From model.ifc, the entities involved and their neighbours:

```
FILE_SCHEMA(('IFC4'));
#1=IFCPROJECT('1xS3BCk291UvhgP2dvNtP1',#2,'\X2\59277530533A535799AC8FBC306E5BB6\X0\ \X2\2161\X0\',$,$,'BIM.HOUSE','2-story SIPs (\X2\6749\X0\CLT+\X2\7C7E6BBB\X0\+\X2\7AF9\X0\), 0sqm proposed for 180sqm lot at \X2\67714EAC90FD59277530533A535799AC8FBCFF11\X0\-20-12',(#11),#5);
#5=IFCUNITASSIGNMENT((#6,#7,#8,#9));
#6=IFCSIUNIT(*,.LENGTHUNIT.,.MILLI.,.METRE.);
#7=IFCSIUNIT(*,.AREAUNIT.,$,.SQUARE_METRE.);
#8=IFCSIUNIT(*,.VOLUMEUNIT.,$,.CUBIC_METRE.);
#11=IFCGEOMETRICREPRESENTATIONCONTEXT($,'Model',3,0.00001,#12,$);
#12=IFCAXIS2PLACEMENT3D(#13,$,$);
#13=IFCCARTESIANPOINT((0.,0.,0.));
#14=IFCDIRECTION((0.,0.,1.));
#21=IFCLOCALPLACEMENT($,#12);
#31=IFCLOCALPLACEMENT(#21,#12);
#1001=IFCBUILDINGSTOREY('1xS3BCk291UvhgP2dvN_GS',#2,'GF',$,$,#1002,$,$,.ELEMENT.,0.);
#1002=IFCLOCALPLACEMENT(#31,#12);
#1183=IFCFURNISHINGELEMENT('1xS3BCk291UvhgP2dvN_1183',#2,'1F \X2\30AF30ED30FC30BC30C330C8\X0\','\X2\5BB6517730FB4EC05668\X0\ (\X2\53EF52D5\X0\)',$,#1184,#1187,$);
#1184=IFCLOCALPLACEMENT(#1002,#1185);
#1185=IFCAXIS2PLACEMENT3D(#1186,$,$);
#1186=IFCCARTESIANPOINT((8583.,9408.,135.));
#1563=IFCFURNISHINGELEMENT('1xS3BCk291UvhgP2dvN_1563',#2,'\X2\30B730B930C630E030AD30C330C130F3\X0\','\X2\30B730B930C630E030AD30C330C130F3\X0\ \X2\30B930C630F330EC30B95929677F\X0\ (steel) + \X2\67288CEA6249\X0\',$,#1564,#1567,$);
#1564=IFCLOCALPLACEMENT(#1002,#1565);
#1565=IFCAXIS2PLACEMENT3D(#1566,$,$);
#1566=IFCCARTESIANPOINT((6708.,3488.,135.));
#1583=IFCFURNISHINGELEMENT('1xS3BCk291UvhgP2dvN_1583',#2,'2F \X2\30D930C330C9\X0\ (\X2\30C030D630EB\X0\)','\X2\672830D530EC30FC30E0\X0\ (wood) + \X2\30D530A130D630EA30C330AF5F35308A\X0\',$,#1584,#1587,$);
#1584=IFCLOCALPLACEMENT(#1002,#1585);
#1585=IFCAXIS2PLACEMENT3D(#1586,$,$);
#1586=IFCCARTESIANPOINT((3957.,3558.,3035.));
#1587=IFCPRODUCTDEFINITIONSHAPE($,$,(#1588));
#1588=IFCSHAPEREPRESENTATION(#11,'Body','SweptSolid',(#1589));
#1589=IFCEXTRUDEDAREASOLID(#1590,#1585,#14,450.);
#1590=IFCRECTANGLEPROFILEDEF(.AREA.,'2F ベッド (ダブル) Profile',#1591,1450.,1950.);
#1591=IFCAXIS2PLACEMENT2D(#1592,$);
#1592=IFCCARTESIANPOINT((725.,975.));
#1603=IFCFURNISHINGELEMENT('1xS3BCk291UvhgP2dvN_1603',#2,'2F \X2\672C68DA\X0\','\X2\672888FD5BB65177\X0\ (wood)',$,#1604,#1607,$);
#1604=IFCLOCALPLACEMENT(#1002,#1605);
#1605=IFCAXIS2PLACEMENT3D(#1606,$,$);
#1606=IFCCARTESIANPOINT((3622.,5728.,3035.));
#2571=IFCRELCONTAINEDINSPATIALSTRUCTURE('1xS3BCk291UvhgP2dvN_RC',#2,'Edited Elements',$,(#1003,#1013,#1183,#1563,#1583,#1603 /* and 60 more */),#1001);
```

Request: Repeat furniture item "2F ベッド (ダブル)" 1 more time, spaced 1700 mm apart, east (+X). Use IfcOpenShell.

```python
import numpy as np
import ifcopenshell
import ifcopenshell.api.geometry
import ifcopenshell.api.root
import ifcopenshell.util.element
import ifcopenshell.util.placement
import ifcopenshell.util.unit

model = ifcopenshell.open("model.ifc")
unit_scale = ifcopenshell.util.unit.calculate_unit_scale(model)


def reuse_history(source, copy):
    """copy_class also copies each property set's owner history, people and application; keep the originals."""
    for rel in copy.IsDefinedBy:
        if rel.is_a("IfcRelDefinesByProperties") and (history := rel.RelatingPropertyDefinition.OwnerHistory):
            rel.RelatingPropertyDefinition.OwnerHistory = source.OwnerHistory
            ifcopenshell.util.element.remove_deep2(model, history)


source = model.by_guid("1xS3BCk291UvhgP2dvN_1583")
base = ifcopenshell.util.placement.get_local_placement(source.ObjectPlacement)
step = np.array([1.0, 0.0, 0.0]) * 1.7 / unit_scale

for i in range(1, 2):
    copy = ifcopenshell.api.root.copy_class(model, product=source)
    copy.Representation = ifcopenshell.util.element.copy_deep(
        model, source.Representation, exclude=["IfcGeometricRepresentationContext", "IfcRepresentationMap"]
    )
    reuse_history(source, copy)
    matrix = base.copy()
    matrix[:3, 3] += i * step
    print("added at", matrix[:3, 3].round(3) + 0.0)
    ifcopenshell.api.geometry.edit_object_placement(model, product=copy, matrix=matrix, is_si=False)

model.write("model_rev.ifc")
```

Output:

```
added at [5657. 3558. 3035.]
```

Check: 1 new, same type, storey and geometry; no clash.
